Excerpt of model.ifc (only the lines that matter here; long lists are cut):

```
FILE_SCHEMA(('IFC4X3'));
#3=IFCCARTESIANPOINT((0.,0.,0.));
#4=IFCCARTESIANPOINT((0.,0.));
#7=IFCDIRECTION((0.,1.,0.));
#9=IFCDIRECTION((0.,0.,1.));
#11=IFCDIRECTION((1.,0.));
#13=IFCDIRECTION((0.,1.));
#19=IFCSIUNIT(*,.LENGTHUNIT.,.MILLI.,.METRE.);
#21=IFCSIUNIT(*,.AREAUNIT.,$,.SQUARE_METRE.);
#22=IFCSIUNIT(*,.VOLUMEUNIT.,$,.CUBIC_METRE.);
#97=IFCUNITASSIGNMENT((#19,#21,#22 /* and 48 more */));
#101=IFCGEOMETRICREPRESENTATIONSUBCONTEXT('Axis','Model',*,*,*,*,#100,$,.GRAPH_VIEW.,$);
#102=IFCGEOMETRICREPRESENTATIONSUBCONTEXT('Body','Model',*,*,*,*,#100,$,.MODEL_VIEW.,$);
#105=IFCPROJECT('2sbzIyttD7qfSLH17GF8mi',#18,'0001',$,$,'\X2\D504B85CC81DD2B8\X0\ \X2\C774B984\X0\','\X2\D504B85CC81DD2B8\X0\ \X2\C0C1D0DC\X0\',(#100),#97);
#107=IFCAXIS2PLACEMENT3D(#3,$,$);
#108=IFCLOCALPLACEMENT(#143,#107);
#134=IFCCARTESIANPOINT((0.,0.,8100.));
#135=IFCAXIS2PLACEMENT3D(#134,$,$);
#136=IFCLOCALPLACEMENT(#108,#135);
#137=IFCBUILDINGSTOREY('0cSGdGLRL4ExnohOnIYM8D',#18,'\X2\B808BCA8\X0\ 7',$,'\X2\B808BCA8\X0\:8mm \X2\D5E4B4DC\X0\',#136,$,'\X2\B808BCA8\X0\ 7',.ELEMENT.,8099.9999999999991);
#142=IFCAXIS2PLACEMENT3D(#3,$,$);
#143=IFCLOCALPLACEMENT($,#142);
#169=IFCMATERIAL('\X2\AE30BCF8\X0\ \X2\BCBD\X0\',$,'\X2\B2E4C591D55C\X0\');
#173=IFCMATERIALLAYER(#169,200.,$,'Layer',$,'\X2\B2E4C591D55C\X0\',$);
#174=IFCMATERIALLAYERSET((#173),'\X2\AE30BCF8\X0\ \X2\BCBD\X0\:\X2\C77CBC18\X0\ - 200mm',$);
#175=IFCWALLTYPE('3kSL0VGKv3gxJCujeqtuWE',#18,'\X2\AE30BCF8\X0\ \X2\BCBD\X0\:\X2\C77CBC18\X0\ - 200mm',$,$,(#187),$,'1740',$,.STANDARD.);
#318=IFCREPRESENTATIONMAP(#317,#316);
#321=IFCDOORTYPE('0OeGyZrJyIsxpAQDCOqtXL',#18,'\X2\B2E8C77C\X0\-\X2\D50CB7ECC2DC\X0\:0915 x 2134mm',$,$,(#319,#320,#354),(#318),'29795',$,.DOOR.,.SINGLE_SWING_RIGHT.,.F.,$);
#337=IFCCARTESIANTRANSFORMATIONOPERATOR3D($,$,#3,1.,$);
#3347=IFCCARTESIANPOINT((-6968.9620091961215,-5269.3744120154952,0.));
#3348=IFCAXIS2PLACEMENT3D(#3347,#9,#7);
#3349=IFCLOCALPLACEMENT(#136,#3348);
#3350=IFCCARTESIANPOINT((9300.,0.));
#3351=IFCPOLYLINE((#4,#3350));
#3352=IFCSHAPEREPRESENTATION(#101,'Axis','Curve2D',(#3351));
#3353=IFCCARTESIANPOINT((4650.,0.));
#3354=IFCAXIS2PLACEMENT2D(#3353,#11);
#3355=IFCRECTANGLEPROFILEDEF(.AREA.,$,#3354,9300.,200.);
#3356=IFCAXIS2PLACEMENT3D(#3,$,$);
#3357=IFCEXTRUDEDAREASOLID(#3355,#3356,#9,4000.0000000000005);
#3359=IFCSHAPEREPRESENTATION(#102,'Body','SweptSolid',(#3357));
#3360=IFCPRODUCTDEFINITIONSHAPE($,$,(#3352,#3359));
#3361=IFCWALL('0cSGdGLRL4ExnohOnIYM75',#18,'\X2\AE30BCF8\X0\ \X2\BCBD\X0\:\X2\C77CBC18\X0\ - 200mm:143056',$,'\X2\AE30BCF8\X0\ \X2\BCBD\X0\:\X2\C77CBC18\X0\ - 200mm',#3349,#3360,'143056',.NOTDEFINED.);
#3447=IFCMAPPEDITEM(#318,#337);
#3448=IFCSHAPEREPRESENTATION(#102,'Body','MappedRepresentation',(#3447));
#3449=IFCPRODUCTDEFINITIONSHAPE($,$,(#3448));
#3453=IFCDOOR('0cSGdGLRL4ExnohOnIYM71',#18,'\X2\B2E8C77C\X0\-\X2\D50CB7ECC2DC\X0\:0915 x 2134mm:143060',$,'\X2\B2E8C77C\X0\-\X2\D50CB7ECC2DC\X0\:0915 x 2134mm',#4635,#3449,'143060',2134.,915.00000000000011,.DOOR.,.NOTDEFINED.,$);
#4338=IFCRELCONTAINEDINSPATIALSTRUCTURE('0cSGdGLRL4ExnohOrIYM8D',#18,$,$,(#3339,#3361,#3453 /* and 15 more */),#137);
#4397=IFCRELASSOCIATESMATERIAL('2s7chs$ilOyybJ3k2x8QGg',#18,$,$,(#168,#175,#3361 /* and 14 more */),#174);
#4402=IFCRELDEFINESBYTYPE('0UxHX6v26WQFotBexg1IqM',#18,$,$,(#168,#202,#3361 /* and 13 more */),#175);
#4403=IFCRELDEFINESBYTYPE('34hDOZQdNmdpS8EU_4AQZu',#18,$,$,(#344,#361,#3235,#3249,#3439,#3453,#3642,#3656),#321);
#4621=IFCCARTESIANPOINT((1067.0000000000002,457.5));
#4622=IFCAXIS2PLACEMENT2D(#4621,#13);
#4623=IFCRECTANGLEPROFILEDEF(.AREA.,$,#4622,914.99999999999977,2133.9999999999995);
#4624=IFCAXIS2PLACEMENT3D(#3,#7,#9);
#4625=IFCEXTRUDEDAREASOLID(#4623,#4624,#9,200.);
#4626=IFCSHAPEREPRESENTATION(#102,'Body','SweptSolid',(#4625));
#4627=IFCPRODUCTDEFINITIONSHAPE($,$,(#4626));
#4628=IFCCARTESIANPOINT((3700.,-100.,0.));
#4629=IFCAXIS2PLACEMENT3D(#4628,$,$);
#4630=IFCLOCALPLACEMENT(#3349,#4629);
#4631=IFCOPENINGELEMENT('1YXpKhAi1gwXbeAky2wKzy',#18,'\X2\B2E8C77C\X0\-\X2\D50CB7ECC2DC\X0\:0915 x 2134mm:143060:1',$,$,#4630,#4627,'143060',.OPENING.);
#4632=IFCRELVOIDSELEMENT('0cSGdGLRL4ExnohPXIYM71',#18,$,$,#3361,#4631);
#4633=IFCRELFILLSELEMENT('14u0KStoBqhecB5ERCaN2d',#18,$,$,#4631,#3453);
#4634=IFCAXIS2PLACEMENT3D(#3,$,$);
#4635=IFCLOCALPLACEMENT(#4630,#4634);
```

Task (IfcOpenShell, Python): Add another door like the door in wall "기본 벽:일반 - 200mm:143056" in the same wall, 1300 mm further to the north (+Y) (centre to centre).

```python
import ifcopenshell
import ifcopenshell.api.feature
import ifcopenshell.api.geometry
import ifcopenshell.api.root
import ifcopenshell.geom
import ifcopenshell.util.element
import ifcopenshell.util.placement
import ifcopenshell.util.shape

model = ifcopenshell.open("model.ifc")
settings = ifcopenshell.geom.settings()


def volume(element):
    """Net volume in cubic metres, openings subtracted."""
    shape = ifcopenshell.geom.create_shape(settings, element)
    return ifcopenshell.util.shape.get_volume(shape.geometry)


def reuse_history(source, copy):
    """copy_class also copies each property set's owner history, people and application; keep the originals."""
    for rel in copy.IsDefinedBy:
        if rel.is_a("IfcRelDefinesByProperties") and (history := rel.RelatingPropertyDefinition.OwnerHistory):
            rel.RelatingPropertyDefinition.OwnerHistory = source.OwnerHistory
            ifcopenshell.util.element.remove_deep2(model, history)


door = model.by_guid("0cSGdGLRL4ExnohOnIYM71")
opening = door.FillsVoids[0].RelatingOpeningElement
wall = opening.VoidsElements[0].RelatingBuildingElement
before = volume(wall)
shift = ifcopenshell.util.placement.get_local_placement(wall.ObjectPlacement)[:3, 0] * 1300.0

# copy_class copies the void relationship, type, container and properties, but no geometry.
new_opening = ifcopenshell.api.root.copy_class(model, product=opening)
new_opening.Representation = ifcopenshell.util.element.copy_deep(
    model, opening.Representation, exclude=["IfcGeometricRepresentationContext", "IfcRepresentationMap"]
)
new_opening.Name = "단일-플러시:0915 x 2134mm"
new_opening.Tag = None
new_door = ifcopenshell.api.root.copy_class(model, product=door)
new_door.Representation = ifcopenshell.util.element.copy_deep(
    model, door.Representation, exclude=["IfcGeometricRepresentationContext", "IfcRepresentationMap"]
)
new_door.Name = "단일-플러시:0915 x 2134mm"
new_door.Tag = None
reuse_history(door, new_door)
ifcopenshell.api.feature.add_filling(model, opening=new_opening, element=new_door)

for old, new in ((opening, new_opening), (door, new_door)):
    matrix = ifcopenshell.util.placement.get_local_placement(old.ObjectPlacement)
    matrix[:3, 3] += shift
    ifcopenshell.api.geometry.edit_object_placement(model, product=new, matrix=matrix, is_si=False)

after = volume(wall)

print(f"wall volume {before:.3f} -> {after:.3f} m3")

model.write("model_edited.ifc")
```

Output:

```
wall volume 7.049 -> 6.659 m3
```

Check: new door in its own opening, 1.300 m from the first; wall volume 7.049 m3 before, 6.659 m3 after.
